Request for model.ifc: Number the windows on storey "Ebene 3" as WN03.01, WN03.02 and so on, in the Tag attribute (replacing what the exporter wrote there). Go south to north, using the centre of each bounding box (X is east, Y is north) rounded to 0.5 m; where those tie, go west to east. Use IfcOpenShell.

First a look at what the model holds.

```python
import ifcopenshell
import ifcopenshell.util.element
import ifcopenshell.util.placement

model = ifcopenshell.open("model.ifc")
print(model.schema)
storey = next(s for s in model.by_type("IfcBuildingStorey") if s.Name == "Ebene 3")
windows = [e for e in ifcopenshell.util.element.get_decomposition(storey) if e.is_a("IfcWindow")]
for e in sorted(windows, key=lambda e: e.id()):
    origin = ifcopenshell.util.placement.get_local_placement(e.ObjectPlacement)[:3, 3]
    print(e.id(), e.Tag, e.Name, origin.round(2) + 0.0, sep=" | ")
```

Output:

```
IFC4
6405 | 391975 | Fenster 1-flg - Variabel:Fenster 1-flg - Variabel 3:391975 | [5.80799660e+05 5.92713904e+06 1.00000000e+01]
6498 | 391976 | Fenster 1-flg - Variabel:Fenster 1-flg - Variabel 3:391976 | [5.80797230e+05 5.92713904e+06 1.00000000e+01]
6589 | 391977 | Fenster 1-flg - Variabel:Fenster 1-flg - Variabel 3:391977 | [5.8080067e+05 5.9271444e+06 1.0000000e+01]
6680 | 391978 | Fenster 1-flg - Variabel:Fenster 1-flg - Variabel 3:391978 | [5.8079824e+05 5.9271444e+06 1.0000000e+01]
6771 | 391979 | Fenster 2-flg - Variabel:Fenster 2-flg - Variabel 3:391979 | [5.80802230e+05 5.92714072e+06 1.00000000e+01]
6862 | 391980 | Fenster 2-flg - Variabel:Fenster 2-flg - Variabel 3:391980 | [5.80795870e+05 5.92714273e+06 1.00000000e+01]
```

```python
import ifcopenshell
import ifcopenshell.geom
import ifcopenshell.util.element
import ifcopenshell.util.shape

model = ifcopenshell.open("model.ifc")
settings = ifcopenshell.geom.settings()
settings.set("use-world-coords", True)


def centre(element):
    shape = ifcopenshell.geom.create_shape(settings, element)
    return ifcopenshell.util.shape.get_bbox_centroid(shape.geometry)


storey = next(s for s in model.by_type("IfcBuildingStorey") if s.Name == "Ebene 3")
windows = [e for e in ifcopenshell.util.element.get_decomposition(storey) if e.is_a("IfcWindow")]

# Insertion points can sit at a corner or the storey origin, so sort by the geometry (in metres).
centres = {e: centre(e) for e in windows}
windows.sort(key=lambda e: (round(centres[e][1] / 0.5), centres[e][0]))

for i, e in enumerate(windows, start=1):
    number = f"WN03.{i:02d}"
    e.Tag = number
    print(e.id(), number)

model.write("model-out.ifc")
```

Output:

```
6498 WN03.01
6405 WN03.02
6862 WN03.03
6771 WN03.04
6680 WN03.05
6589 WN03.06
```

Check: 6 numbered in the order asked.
